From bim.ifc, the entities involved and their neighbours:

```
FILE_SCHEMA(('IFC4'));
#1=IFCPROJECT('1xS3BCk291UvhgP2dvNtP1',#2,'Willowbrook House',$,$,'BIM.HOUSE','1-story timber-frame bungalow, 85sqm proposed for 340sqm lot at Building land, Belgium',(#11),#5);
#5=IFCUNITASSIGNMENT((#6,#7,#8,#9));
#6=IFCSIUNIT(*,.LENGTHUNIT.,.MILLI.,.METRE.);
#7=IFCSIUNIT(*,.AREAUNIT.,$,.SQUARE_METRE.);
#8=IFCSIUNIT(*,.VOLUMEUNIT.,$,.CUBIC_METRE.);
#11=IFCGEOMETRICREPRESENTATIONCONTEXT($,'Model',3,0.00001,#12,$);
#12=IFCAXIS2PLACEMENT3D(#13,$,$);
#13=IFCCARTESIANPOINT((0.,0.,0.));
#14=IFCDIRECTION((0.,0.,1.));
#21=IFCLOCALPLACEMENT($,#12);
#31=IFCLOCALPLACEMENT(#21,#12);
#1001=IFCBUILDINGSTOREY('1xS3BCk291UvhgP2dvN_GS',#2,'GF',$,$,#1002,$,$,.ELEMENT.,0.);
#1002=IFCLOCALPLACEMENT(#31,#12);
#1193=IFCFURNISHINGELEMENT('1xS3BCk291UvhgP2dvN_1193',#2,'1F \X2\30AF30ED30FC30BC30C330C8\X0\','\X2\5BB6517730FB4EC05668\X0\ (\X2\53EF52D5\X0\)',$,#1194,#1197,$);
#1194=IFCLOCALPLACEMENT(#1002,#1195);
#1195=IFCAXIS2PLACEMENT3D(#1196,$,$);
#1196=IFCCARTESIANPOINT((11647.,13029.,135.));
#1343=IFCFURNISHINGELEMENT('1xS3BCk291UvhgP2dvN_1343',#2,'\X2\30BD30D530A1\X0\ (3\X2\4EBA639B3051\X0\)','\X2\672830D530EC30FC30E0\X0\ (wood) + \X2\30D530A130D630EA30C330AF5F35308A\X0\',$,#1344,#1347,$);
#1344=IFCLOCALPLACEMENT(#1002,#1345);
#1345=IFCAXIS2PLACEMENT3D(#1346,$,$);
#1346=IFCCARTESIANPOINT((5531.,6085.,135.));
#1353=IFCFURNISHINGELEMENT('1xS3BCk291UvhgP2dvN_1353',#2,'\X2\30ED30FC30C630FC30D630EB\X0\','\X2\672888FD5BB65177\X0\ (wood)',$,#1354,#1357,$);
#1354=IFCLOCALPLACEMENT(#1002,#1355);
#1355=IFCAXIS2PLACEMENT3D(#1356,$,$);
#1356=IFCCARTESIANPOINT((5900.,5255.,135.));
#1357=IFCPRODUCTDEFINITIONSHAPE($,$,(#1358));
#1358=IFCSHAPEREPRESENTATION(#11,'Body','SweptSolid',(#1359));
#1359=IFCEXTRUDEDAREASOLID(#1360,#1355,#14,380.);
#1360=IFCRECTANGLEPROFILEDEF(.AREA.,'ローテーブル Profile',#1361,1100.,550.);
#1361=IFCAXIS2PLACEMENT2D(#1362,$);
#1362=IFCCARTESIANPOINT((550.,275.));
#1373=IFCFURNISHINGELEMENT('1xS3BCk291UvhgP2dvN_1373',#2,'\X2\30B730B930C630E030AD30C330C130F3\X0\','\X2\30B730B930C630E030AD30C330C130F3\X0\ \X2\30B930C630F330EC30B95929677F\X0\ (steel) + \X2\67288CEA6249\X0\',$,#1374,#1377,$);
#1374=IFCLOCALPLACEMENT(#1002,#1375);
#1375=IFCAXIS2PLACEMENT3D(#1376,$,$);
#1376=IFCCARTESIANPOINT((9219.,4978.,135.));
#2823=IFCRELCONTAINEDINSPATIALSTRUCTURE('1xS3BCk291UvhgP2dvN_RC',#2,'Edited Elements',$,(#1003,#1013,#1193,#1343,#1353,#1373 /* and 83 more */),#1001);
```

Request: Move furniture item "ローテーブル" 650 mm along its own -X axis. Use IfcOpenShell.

```python
import ifcopenshell
import ifcopenshell.api.geometry
import ifcopenshell.util.placement
import ifcopenshell.util.unit

model = ifcopenshell.open("bim.ifc")
unit_scale = ifcopenshell.util.unit.calculate_unit_scale(model)

item = model.by_guid("1xS3BCk291UvhgP2dvN_1353")
matrix = ifcopenshell.util.placement.get_local_placement(item.ObjectPlacement)
matrix[:3, 3] -= matrix[:3, 0] * 0.65 / unit_scale
ifcopenshell.api.geometry.edit_object_placement(model, product=item, matrix=matrix, is_si=False)

print(ifcopenshell.util.placement.get_local_placement(item.ObjectPlacement).round(3) + 0.0)

model.write("bim_rev.ifc")
```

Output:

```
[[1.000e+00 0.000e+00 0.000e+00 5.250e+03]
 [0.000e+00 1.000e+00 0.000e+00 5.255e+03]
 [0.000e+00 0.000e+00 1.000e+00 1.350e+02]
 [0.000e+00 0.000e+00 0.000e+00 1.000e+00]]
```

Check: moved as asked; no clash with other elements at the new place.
